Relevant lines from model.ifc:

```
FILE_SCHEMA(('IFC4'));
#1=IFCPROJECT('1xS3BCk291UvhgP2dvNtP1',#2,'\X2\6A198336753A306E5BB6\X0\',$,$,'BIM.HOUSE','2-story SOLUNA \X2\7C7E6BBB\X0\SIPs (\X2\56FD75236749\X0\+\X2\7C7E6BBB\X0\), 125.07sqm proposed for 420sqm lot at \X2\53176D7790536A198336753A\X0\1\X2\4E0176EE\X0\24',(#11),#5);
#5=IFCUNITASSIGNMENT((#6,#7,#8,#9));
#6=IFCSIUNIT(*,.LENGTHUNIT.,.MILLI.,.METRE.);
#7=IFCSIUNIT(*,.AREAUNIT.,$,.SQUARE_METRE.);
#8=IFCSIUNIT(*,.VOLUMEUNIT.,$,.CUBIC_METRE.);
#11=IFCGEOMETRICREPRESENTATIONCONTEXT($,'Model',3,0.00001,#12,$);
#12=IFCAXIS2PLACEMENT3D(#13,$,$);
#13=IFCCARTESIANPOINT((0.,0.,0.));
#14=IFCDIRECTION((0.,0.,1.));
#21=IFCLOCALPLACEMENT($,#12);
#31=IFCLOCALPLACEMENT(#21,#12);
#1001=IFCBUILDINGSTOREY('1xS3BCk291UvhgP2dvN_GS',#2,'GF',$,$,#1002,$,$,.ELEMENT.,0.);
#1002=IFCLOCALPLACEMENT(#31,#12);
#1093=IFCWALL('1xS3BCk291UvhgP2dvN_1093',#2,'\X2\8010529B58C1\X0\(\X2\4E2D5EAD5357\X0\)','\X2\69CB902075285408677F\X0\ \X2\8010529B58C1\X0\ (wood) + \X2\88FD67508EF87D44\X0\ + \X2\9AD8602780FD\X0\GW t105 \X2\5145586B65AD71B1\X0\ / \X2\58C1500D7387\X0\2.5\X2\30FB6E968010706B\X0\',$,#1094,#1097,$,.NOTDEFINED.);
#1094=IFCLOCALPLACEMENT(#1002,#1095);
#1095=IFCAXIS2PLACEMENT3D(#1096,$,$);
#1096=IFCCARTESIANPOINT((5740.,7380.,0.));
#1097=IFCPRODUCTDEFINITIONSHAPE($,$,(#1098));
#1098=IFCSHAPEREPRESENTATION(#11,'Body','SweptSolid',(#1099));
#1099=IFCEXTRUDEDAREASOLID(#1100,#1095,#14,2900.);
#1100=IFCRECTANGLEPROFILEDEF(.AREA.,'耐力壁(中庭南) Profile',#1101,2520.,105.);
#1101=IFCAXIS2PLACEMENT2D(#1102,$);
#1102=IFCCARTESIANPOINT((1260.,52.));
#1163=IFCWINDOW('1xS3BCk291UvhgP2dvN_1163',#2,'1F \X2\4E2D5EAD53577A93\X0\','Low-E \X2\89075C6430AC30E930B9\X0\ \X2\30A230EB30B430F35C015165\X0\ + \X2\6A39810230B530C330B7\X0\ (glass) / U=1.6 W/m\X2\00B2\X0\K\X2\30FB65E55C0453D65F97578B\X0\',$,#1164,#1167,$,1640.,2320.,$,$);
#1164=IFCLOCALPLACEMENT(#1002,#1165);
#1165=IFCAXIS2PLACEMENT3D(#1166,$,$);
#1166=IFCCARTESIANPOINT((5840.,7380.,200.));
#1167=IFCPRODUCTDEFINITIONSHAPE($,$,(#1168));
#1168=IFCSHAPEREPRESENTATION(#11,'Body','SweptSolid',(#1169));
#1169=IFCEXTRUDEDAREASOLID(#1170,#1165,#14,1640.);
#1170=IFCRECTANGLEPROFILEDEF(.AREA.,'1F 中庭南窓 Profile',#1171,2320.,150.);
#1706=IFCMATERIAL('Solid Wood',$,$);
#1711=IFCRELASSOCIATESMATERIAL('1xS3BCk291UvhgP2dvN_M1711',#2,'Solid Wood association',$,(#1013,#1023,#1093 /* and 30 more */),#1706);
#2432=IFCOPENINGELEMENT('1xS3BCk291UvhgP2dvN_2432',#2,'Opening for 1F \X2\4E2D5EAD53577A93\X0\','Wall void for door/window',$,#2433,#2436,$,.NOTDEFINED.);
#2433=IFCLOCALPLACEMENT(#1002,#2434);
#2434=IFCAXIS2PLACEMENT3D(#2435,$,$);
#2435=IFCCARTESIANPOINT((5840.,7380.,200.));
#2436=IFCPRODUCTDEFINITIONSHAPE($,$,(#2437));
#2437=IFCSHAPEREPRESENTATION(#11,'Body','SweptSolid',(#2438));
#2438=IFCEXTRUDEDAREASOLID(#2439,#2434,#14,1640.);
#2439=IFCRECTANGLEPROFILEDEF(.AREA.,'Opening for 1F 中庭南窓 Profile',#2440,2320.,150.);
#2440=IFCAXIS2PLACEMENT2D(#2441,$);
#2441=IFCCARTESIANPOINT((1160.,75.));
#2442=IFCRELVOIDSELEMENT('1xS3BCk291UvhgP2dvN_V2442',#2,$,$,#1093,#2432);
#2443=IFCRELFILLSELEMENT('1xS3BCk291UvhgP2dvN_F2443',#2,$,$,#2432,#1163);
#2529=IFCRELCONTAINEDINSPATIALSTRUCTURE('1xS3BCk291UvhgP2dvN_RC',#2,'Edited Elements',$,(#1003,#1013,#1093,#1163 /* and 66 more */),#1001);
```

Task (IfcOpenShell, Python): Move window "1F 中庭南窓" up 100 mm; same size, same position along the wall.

```python
import numpy as np
import ifcopenshell
import ifcopenshell.api.geometry
import ifcopenshell.util.placement
import ifcopenshell.util.unit

model = ifcopenshell.open("model.ifc")
unit_scale = ifcopenshell.util.unit.calculate_unit_scale(model)

window = model.by_guid("1xS3BCk291UvhgP2dvN_1163")
opening = window.FillsVoids[0].RelatingOpeningElement
dz = 100.0

shift = np.array([0.0, 0.0, dz])
# The window is not placed relative to its opening, so move both.
for product in (opening, window):
    matrix = ifcopenshell.util.placement.get_local_placement(product.ObjectPlacement)
    matrix[:3, 3] += shift
    ifcopenshell.api.geometry.edit_object_placement(model, product=product, matrix=matrix, is_si=False)

print(f"moved by {dz * unit_scale:+.3f} m")

model.write("model_updated.ifc")
```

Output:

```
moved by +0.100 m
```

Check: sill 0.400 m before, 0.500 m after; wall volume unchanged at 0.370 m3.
